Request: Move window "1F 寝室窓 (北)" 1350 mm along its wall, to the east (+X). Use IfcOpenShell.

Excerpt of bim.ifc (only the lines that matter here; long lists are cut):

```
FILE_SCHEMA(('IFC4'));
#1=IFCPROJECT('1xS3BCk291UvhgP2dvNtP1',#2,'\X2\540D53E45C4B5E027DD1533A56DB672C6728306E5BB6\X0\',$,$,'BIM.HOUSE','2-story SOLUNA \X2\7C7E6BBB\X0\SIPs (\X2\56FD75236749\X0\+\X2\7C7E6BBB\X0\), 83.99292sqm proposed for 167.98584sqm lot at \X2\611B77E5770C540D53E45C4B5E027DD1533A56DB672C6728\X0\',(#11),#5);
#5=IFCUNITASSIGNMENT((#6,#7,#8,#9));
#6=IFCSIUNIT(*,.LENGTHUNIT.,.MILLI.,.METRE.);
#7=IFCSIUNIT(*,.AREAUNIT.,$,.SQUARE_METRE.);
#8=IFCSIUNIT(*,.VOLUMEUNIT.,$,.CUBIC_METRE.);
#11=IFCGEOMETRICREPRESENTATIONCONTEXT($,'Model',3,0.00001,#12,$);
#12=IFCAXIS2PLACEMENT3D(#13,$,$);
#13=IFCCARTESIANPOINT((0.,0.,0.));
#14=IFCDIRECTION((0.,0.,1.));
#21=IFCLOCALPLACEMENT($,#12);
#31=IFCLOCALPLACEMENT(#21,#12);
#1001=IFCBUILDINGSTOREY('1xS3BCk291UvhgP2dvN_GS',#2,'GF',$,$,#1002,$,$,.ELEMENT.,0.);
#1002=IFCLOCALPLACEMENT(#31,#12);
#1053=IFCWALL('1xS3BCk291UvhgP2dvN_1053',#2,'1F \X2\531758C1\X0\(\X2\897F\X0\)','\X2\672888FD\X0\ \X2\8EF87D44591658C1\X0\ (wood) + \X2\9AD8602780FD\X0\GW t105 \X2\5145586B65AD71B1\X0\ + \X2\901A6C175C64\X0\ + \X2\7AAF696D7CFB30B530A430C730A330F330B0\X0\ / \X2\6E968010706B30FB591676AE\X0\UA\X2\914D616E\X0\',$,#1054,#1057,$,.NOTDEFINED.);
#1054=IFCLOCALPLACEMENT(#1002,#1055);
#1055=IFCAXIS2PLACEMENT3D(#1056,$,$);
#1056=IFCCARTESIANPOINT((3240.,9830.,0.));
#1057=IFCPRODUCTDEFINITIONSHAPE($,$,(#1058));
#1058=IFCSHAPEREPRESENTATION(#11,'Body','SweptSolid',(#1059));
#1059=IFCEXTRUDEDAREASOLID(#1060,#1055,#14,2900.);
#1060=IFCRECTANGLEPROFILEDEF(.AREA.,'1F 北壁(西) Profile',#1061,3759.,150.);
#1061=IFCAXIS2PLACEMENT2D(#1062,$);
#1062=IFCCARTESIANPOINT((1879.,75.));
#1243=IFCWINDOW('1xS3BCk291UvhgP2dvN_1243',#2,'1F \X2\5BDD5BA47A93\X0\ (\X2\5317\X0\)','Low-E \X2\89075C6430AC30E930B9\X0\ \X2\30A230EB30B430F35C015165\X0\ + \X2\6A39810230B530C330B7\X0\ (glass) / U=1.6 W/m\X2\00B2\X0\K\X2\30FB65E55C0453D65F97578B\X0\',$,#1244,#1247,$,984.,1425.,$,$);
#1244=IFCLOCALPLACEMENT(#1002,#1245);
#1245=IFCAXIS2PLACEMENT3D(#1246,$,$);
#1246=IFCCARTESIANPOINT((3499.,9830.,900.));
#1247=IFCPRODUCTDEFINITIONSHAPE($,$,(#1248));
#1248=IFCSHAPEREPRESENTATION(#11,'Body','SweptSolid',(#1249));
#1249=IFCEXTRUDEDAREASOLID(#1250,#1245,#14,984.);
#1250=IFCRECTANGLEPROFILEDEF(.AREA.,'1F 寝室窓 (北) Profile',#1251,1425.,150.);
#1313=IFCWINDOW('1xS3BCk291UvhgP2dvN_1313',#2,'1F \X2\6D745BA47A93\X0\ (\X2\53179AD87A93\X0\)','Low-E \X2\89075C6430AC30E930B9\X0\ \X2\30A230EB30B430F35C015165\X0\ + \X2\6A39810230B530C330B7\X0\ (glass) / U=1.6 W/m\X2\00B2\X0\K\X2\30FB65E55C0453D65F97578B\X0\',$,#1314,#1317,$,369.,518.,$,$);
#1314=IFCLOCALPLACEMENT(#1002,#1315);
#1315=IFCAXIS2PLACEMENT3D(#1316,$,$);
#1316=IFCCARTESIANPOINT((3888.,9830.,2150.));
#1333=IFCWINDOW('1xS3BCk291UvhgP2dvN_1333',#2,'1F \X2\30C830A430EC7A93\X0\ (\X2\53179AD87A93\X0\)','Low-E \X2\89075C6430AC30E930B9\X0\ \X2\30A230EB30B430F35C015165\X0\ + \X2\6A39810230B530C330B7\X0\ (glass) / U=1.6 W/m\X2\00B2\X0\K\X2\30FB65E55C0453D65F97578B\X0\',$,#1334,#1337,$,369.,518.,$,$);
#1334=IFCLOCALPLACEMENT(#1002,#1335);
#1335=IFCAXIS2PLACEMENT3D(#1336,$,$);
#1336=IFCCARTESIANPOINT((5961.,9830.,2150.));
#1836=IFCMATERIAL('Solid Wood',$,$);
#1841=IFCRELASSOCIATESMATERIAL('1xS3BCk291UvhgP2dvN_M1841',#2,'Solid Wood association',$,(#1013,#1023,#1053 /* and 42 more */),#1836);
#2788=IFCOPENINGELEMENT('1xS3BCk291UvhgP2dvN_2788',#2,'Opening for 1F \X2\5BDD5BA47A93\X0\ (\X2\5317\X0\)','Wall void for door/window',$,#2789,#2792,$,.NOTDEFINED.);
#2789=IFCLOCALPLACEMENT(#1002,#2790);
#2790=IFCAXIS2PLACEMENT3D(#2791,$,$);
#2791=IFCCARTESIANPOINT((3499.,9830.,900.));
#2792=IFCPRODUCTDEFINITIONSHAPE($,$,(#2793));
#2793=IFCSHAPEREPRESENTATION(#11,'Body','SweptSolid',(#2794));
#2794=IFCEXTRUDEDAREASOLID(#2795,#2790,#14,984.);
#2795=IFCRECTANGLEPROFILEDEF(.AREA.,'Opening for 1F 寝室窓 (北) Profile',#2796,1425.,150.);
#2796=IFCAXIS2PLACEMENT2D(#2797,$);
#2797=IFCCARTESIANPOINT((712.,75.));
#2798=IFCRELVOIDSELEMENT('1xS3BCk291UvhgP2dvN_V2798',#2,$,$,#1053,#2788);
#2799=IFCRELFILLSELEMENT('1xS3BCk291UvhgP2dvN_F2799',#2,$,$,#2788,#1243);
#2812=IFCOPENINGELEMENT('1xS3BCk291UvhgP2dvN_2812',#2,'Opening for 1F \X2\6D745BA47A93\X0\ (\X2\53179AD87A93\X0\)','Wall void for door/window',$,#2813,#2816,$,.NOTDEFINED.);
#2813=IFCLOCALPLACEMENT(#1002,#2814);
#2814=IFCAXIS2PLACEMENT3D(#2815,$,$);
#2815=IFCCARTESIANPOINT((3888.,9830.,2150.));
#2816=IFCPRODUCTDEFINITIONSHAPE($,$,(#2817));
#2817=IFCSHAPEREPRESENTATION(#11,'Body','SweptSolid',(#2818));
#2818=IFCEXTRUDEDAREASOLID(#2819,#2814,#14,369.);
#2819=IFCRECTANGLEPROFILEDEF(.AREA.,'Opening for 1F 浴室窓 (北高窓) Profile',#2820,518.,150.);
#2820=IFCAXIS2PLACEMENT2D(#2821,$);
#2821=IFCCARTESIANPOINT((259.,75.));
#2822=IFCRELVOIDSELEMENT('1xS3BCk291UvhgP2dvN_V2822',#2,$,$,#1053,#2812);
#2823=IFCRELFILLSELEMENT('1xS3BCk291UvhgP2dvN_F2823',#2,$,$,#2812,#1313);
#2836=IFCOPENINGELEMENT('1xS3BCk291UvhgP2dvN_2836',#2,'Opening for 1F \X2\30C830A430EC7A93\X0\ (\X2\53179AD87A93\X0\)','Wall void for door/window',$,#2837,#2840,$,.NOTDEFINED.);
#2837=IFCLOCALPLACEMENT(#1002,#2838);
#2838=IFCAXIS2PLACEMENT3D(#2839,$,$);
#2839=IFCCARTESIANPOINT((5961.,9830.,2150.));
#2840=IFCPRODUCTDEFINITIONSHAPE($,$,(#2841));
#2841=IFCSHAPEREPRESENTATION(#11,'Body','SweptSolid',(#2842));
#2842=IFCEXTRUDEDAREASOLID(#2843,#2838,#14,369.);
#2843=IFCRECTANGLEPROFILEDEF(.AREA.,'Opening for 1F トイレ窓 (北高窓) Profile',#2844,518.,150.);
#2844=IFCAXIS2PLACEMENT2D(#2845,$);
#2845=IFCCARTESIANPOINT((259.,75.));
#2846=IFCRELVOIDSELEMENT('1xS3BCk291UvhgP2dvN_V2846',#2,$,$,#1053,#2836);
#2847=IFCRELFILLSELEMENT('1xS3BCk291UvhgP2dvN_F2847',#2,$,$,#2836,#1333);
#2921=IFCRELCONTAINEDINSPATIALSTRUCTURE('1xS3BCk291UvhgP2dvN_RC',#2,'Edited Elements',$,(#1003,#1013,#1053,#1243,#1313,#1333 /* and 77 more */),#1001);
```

```python
import ifcopenshell
import ifcopenshell.api.geometry
import ifcopenshell.util.placement
import ifcopenshell.util.unit

model = ifcopenshell.open("bim.ifc")
unit_scale = ifcopenshell.util.unit.calculate_unit_scale(model)

window = model.by_id(1243)
opening = window.FillsVoids[0].RelatingOpeningElement
wall = opening.VoidsElements[0].RelatingBuildingElement

wall_matrix = ifcopenshell.util.placement.get_local_placement(wall.ObjectPlacement)
shift = wall_matrix[:3, 0] * 1.35 / unit_scale
before = ifcopenshell.util.placement.get_local_placement(window.ObjectPlacement)[:3, 3].copy()

# The window is not placed relative to its opening, so move both.
for product in (opening, window):
    matrix = ifcopenshell.util.placement.get_local_placement(product.ObjectPlacement)
    matrix[:3, 3] += shift
    ifcopenshell.api.geometry.edit_object_placement(model, product=product, matrix=matrix, is_si=False)

after = ifcopenshell.util.placement.get_local_placement(window.ObjectPlacement)[:3, 3]
print("window moved by", (after - before).round(3) + 0.0)

model.write("bim_edited.ifc")
```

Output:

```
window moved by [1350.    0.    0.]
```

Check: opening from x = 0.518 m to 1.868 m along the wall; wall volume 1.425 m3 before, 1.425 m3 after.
